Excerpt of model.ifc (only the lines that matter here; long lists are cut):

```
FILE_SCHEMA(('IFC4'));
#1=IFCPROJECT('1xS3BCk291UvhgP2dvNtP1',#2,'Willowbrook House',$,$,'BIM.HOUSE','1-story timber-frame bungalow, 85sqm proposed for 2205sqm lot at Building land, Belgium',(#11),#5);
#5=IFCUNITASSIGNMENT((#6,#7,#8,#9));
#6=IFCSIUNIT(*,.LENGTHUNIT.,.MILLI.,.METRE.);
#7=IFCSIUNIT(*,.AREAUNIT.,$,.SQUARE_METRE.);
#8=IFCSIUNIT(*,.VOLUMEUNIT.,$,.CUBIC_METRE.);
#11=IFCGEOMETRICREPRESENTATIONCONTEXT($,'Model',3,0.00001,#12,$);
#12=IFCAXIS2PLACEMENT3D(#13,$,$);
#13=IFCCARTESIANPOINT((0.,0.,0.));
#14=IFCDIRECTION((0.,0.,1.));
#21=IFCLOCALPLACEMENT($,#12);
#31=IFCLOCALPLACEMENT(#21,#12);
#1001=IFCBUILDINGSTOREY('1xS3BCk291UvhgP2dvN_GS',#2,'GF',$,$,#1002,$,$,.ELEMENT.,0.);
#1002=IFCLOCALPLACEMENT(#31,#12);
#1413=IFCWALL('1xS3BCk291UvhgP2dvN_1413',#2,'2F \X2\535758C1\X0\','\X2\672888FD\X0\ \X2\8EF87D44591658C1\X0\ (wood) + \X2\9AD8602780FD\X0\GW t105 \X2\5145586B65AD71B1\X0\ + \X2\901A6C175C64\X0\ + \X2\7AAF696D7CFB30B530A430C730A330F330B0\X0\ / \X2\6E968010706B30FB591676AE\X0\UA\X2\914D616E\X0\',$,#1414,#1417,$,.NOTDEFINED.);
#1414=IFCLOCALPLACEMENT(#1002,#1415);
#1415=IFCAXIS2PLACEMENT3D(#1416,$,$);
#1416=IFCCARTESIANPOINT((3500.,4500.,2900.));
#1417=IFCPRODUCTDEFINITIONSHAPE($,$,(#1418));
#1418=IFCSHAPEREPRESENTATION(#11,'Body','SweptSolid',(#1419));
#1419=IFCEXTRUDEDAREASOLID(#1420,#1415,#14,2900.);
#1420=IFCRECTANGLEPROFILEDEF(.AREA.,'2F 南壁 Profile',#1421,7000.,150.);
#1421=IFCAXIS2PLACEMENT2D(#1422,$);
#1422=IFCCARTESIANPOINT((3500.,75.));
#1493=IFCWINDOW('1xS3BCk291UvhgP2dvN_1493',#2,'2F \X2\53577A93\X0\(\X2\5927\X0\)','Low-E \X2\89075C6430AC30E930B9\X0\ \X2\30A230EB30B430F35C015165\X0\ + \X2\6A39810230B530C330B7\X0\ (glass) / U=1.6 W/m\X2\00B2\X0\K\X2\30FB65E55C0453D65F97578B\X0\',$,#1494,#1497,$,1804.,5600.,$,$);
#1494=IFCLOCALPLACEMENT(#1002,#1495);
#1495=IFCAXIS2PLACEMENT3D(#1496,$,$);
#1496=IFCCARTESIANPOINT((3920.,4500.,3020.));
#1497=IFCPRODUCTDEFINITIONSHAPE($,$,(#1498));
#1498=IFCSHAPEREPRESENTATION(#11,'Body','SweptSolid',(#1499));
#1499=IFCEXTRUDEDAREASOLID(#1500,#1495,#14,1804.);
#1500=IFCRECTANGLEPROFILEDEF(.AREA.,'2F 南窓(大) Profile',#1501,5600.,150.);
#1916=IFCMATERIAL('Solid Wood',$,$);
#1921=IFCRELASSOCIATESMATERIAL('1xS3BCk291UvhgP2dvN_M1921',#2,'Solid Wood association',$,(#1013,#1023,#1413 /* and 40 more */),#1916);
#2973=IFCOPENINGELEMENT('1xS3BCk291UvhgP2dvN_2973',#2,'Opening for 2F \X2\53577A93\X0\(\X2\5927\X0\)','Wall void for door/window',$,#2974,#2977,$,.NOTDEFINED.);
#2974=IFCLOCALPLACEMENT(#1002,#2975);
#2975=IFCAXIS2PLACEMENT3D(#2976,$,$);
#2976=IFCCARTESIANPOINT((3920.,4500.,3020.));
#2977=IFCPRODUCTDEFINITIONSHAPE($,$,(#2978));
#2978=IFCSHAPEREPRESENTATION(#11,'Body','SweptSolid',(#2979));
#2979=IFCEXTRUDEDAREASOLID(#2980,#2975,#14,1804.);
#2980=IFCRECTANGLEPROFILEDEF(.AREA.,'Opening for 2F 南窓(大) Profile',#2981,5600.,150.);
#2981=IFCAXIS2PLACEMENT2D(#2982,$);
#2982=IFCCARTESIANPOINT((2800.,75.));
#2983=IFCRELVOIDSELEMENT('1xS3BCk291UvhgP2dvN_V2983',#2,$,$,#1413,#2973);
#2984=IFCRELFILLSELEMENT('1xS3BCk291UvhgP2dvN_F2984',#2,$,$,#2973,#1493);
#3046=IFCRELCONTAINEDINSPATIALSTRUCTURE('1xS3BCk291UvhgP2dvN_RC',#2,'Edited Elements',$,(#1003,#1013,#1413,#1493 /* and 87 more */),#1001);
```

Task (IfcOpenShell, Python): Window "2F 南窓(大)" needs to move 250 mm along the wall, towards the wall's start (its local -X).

```python
import ifcopenshell
import ifcopenshell.api.geometry
import ifcopenshell.util.placement

model = ifcopenshell.open("model.ifc")

window = model.by_guid("1xS3BCk291UvhgP2dvN_1493")
opening = window.FillsVoids[0].RelatingOpeningElement
wall = opening.VoidsElements[0].RelatingBuildingElement

wall_matrix = ifcopenshell.util.placement.get_local_placement(wall.ObjectPlacement)
shift = wall_matrix[:3, 0] * -250.0
before = ifcopenshell.util.placement.get_local_placement(window.ObjectPlacement)[:3, 3].copy()

# The window is not placed relative to its opening, so move both.
for product in (opening, window):
    matrix = ifcopenshell.util.placement.get_local_placement(product.ObjectPlacement)
    matrix[:3, 3] += shift
    ifcopenshell.api.geometry.edit_object_placement(model, product=product, matrix=matrix, is_si=False)

after = ifcopenshell.util.placement.get_local_placement(window.ObjectPlacement)[:3, 3]
print("window moved by", (after - before).round(3) + 0.0)

model.write("model_updated.ifc")
```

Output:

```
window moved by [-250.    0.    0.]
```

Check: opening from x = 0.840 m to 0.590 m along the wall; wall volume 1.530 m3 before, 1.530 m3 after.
